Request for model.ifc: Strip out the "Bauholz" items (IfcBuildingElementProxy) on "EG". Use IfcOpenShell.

First a look at what the model holds.

```python
import ifcopenshell
import ifcopenshell.util.element

model = ifcopenshell.open("model.ifc")
print(model.schema)
storey = next(s for s in model.by_type("IfcBuildingStorey") if s.Name == "EG")
proxies = [e for e in ifcopenshell.util.element.get_decomposition(storey) if e.is_a("IfcBuildingElementProxy")]
seen = {}
for e in proxies:
    element_type = ifcopenshell.util.element.get_type(e)
    name = element_type.Name if element_type not in (None, e) else None
    seen[name] = seen.get(name, 0) + 1
for name, count in sorted(seen.items(), key=str):
    print(count, "x", name)
```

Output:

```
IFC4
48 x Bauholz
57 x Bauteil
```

```python
import ifcopenshell
import ifcopenshell.api.root
import ifcopenshell.util.element

model = ifcopenshell.open("model.ifc")

storey = next(s for s in model.by_type("IfcBuildingStorey") if s.Name == "EG")
proxies = [e for e in ifcopenshell.util.element.get_decomposition(storey) if e.is_a("IfcBuildingElementProxy")]
targets = [e for e in proxies if (t := ifcopenshell.util.element.get_type(e)) not in (None, e) and t.Name == "Bauholz"]

for e in targets:
    ifcopenshell.api.root.remove_product(model, product=e)
print(len(targets), "removed")

model.write("model_rev.ifc")
```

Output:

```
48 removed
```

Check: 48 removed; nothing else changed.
